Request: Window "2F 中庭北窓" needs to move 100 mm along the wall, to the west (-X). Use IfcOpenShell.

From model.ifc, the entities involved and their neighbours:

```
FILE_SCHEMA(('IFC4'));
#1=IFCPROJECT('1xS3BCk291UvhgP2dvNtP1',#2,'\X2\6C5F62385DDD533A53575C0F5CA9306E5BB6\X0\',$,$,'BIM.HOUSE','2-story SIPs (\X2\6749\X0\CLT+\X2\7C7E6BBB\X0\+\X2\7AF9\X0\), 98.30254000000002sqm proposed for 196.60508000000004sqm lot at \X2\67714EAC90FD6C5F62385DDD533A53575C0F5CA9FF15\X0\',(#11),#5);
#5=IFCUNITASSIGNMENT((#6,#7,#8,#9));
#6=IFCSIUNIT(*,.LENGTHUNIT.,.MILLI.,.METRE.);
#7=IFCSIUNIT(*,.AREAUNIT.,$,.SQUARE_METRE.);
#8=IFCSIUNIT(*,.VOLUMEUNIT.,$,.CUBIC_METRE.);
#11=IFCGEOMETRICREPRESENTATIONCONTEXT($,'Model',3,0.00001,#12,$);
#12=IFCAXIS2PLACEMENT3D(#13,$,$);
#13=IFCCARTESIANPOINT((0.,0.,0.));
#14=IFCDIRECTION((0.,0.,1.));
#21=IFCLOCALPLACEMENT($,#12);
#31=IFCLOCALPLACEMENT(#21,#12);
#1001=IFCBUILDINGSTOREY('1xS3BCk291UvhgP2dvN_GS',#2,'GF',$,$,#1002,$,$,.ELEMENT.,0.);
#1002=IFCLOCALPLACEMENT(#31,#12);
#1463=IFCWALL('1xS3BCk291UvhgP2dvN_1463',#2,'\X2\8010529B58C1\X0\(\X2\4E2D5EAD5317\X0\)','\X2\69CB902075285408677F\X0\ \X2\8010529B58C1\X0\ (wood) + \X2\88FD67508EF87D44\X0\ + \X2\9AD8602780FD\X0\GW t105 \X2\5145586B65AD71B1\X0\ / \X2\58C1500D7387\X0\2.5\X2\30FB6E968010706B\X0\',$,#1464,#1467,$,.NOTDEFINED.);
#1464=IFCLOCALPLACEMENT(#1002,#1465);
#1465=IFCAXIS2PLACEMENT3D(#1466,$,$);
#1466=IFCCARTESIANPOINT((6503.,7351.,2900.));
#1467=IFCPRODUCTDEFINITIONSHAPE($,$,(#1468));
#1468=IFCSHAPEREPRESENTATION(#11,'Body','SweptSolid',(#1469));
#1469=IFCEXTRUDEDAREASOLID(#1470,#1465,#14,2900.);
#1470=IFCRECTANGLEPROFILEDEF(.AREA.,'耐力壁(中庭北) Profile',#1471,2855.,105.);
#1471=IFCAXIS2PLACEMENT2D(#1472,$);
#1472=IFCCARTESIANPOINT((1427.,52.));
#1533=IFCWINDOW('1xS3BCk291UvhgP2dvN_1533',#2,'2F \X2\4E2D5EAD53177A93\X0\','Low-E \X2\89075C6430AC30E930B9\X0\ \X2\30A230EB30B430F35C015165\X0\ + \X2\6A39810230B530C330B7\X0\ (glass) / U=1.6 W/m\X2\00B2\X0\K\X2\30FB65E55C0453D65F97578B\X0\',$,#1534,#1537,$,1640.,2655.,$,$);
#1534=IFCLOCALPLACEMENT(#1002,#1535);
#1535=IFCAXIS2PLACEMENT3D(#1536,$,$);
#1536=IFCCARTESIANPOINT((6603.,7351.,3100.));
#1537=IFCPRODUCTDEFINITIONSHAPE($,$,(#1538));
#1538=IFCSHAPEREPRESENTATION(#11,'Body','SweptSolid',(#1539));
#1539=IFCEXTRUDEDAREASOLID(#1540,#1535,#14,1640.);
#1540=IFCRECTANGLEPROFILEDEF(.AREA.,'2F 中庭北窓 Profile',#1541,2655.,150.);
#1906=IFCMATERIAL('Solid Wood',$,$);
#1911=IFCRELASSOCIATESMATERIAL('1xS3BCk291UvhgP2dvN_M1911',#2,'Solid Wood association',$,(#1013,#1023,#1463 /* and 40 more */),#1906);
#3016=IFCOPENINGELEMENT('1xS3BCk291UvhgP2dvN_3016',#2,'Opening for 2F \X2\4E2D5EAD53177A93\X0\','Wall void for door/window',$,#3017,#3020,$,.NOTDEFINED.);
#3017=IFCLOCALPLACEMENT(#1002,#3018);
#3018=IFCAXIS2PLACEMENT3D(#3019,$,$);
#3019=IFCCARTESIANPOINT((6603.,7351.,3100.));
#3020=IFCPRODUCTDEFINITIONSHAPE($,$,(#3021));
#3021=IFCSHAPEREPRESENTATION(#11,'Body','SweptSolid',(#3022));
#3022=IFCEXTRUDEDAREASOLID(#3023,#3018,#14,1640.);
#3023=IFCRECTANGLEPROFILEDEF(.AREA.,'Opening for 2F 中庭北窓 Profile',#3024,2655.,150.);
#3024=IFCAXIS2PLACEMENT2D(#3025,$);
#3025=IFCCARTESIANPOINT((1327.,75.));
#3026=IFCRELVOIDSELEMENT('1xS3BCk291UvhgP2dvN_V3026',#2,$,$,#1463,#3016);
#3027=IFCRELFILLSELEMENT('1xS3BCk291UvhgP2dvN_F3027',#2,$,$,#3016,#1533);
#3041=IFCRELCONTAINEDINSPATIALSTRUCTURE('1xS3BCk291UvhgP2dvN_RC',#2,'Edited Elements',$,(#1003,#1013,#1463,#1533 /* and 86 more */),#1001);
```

```python
import ifcopenshell
import ifcopenshell.api.geometry
import ifcopenshell.util.placement

model = ifcopenshell.open("model.ifc")

window = model.by_guid("1xS3BCk291UvhgP2dvN_1533")
opening = window.FillsVoids[0].RelatingOpeningElement
wall = opening.VoidsElements[0].RelatingBuildingElement

wall_matrix = ifcopenshell.util.placement.get_local_placement(wall.ObjectPlacement)
shift = wall_matrix[:3, 0] * -100.0
before = ifcopenshell.util.placement.get_local_placement(window.ObjectPlacement)[:3, 3].copy()

# The window is not placed relative to its opening, so move both.
for product in (opening, window):
    matrix = ifcopenshell.util.placement.get_local_placement(product.ObjectPlacement)
    matrix[:3, 3] += shift
    ifcopenshell.api.geometry.edit_object_placement(model, product=product, matrix=matrix, is_si=False)

after = ifcopenshell.util.placement.get_local_placement(window.ObjectPlacement)[:3, 3]
print("window moved by", (after - before).round(3) + 0.0)

model.write("model_updated.ifc")
```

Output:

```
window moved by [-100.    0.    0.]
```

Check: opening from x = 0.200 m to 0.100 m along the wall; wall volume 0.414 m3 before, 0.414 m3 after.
